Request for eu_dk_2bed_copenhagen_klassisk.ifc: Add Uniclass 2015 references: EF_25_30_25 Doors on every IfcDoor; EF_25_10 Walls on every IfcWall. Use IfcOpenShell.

First a look at what the model holds.

```python
import ifcopenshell

model = ifcopenshell.open("eu_dk_2bed_copenhagen_klassisk.ifc")
print(model.schema)
print("classifications:", [c.Name for c in model.by_type("IfcClassification")])
for ifc_class in ("IfcDoor", "IfcRoof", "IfcStair", "IfcWall", "IfcWindow"):
    print(ifc_class, len(model.by_type(ifc_class)))
```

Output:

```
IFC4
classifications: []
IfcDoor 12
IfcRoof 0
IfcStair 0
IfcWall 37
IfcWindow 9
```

```python
import ifcopenshell
import ifcopenshell.api.classification

model = ifcopenshell.open("eu_dk_2bed_copenhagen_klassisk.ifc")

system = ifcopenshell.api.classification.add_classification(model, classification="Uniclass 2015")

codes = {
    "IfcDoor": ("EF_25_30_25", "Doors"),
    "IfcWall": ("EF_25_10", "Walls"),
}
for ifc_class, (code, name) in codes.items():
    products = model.by_type(ifc_class)
    ifcopenshell.api.classification.add_reference(
        model, products=products, classification=system, identification=code, name=name
    )
    print(code, len(products))

model.write("eu_dk_2bed_copenhagen_klassisk_edited.ifc")
```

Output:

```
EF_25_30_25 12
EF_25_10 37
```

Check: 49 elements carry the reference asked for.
